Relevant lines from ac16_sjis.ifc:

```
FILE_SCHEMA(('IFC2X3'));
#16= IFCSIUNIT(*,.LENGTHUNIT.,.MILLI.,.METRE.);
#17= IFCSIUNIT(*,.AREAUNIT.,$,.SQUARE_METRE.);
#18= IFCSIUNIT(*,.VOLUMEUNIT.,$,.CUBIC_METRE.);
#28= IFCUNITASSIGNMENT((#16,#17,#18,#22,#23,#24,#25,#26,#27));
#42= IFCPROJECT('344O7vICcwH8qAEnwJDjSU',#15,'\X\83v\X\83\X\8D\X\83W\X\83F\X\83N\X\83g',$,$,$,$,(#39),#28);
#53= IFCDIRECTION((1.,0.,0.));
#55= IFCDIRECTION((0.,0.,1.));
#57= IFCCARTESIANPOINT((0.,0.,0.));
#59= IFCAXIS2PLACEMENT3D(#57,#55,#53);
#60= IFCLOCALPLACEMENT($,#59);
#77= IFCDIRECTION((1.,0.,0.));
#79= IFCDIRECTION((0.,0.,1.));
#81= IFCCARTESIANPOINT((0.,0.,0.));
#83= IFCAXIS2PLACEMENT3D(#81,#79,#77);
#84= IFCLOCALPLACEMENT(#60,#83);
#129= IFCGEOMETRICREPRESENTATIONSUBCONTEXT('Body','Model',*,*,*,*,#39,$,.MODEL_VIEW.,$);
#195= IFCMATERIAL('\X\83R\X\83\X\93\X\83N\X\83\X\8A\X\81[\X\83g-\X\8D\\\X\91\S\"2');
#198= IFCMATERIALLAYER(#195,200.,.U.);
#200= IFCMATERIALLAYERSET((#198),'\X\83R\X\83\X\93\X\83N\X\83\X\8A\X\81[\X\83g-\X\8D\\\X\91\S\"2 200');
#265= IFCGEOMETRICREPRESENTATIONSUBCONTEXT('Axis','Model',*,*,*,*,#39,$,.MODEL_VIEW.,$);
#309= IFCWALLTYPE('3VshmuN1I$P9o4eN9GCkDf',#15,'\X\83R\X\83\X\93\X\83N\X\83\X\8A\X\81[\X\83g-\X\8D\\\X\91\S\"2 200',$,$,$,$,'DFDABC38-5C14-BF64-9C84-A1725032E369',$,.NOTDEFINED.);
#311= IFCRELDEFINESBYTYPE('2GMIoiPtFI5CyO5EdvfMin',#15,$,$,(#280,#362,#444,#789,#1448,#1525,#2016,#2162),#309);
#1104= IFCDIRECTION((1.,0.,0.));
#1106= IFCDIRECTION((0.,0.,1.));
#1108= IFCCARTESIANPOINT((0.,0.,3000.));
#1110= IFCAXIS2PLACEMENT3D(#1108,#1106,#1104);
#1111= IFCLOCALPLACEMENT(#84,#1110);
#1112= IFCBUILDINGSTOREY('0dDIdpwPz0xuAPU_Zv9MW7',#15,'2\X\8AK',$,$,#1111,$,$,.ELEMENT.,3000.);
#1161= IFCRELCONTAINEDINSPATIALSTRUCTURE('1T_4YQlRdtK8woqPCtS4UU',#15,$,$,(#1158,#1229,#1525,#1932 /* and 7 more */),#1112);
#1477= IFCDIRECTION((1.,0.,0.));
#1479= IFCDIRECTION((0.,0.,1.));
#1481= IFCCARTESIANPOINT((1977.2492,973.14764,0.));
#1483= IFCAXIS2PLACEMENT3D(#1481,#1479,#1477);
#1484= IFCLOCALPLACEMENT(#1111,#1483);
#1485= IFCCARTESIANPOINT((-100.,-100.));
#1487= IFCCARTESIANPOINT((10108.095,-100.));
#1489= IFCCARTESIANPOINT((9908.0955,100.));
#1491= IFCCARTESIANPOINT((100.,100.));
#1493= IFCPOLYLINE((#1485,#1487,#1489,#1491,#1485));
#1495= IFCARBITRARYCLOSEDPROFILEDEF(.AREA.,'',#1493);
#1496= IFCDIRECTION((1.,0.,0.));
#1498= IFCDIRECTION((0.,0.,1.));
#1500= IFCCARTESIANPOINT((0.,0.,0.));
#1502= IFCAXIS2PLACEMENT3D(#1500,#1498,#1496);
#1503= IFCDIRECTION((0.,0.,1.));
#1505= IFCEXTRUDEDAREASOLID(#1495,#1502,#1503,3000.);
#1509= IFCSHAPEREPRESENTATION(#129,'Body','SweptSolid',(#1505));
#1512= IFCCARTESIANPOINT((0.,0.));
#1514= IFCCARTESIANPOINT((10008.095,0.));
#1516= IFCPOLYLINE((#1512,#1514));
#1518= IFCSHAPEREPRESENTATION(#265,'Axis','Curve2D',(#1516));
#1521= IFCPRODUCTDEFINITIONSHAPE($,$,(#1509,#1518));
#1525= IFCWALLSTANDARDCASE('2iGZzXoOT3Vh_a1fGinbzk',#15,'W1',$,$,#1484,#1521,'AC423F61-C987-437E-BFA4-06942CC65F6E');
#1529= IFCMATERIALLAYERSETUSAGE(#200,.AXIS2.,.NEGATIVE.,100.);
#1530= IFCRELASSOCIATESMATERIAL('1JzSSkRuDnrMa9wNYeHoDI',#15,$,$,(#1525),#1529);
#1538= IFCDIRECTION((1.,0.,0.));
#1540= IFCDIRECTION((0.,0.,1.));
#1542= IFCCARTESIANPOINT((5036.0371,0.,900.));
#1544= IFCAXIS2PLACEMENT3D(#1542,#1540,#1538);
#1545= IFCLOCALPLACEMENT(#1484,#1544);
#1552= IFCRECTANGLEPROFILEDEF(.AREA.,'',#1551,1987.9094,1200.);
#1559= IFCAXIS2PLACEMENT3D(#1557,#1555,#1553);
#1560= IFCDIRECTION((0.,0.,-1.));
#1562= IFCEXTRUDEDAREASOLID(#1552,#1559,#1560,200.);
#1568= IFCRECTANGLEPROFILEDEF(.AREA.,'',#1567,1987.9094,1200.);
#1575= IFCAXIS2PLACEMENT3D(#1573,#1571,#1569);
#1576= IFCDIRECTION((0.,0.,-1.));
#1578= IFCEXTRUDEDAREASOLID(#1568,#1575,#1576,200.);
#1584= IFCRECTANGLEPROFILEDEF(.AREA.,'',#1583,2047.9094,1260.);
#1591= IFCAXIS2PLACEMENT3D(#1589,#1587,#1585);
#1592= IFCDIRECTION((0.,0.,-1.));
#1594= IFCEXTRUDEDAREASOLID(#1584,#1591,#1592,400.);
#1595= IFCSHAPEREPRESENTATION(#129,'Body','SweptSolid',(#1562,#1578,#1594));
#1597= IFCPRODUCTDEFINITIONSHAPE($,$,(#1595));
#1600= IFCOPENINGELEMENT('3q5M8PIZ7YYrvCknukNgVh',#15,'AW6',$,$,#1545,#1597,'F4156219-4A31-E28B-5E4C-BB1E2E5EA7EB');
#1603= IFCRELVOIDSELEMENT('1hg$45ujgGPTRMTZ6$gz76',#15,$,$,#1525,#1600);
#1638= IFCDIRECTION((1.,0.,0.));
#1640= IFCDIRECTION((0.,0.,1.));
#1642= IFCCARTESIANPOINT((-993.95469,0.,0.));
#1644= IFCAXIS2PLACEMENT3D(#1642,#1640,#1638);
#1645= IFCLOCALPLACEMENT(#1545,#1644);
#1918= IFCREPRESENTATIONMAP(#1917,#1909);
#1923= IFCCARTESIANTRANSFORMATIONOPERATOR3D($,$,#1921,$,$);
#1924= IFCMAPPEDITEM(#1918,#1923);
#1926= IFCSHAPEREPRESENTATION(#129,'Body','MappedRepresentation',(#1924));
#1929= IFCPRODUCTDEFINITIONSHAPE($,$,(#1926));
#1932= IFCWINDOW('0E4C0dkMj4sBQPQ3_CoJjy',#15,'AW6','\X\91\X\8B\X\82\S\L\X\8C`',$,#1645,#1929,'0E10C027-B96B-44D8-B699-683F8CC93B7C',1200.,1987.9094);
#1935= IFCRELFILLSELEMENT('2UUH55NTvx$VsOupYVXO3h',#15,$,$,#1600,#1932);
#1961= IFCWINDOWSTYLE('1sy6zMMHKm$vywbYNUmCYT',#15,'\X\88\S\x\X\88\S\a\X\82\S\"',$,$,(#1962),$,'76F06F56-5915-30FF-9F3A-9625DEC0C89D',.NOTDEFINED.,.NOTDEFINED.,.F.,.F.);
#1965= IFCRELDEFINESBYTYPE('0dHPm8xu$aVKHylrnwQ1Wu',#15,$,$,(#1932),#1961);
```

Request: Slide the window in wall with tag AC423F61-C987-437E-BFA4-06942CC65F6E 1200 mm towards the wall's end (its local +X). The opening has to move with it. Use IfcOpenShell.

```python
import ifcopenshell
import ifcopenshell.api.geometry
import ifcopenshell.util.placement
import ifcopenshell.util.unit

model = ifcopenshell.open("ac16_sjis.ifc")
unit_scale = ifcopenshell.util.unit.calculate_unit_scale(model)

window = model.by_guid("0E4C0dkMj4sBQPQ3_CoJjy")
opening = window.FillsVoids[0].RelatingOpeningElement
wall = opening.VoidsElements[0].RelatingBuildingElement

wall_matrix = ifcopenshell.util.placement.get_local_placement(wall.ObjectPlacement)
shift = wall_matrix[:3, 0] * 1.2 / unit_scale
before = ifcopenshell.util.placement.get_local_placement(window.ObjectPlacement)[:3, 3].copy()

# The window is placed relative to its opening, so it follows when the opening moves.
matrix = ifcopenshell.util.placement.get_local_placement(opening.ObjectPlacement)
matrix[:3, 3] += shift
ifcopenshell.api.geometry.edit_object_placement(
    model, product=opening, matrix=matrix, is_si=False, should_transform_children=True
)

after = ifcopenshell.util.placement.get_local_placement(window.ObjectPlacement)[:3, 3]
print("window moved by", (after - before).round(3) + 0.0)

model.write("ac16_sjis-out.ifc")
```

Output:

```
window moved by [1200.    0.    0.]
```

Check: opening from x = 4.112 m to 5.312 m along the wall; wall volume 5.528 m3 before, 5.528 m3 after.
